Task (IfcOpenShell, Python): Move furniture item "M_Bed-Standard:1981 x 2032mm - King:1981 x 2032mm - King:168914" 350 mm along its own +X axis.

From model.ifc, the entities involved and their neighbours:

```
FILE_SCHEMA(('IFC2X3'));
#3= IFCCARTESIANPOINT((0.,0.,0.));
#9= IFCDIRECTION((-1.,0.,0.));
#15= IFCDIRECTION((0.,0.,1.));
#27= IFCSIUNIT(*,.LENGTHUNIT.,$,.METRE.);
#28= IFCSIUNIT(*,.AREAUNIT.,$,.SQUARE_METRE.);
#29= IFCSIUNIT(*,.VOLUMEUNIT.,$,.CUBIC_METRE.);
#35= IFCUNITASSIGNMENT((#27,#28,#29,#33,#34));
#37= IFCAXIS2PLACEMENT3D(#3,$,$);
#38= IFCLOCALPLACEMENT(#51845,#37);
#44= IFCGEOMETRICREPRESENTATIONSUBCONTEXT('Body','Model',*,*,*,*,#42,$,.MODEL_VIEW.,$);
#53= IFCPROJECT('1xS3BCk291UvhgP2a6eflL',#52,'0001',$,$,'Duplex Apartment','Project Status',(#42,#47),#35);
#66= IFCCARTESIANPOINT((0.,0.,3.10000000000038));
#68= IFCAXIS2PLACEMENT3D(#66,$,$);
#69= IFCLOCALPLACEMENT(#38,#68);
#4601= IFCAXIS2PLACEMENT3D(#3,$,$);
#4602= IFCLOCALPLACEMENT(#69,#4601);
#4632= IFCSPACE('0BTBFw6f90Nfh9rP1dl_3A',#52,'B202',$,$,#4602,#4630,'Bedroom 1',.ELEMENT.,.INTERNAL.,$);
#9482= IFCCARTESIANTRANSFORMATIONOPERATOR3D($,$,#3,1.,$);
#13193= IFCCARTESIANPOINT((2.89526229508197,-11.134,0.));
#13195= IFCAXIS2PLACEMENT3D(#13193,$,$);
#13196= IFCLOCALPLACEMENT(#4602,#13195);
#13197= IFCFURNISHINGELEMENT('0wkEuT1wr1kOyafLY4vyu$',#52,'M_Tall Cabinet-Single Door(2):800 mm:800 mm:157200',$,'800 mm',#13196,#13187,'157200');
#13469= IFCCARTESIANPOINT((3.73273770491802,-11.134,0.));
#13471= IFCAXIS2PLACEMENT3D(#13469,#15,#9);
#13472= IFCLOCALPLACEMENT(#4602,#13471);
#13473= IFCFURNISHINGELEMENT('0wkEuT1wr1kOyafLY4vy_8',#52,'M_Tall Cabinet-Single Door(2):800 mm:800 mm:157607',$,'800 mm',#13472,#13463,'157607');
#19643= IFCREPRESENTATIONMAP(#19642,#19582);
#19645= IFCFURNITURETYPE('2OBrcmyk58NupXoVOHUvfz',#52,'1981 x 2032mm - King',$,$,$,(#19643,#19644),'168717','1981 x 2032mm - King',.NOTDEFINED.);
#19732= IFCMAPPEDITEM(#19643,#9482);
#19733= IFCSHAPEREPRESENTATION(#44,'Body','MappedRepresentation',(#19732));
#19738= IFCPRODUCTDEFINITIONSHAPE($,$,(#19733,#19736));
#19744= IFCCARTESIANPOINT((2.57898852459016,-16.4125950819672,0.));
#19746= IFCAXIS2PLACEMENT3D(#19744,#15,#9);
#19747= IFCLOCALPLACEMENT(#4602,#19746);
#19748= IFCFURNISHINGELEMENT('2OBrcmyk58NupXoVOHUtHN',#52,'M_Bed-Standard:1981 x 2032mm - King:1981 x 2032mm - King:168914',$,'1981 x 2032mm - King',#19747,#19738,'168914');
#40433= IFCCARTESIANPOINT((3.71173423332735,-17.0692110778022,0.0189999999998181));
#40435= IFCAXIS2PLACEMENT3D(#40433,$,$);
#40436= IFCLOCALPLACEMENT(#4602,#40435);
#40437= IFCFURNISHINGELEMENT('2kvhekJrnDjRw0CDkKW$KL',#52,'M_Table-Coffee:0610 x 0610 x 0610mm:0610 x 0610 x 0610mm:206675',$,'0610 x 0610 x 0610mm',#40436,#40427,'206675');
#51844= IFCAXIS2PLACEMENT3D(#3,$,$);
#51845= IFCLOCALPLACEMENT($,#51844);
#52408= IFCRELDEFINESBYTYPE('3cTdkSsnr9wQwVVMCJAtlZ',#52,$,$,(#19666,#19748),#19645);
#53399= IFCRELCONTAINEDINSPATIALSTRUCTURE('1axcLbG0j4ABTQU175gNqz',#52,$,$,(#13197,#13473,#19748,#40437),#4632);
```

```python
import ifcopenshell
import ifcopenshell.api.geometry
import ifcopenshell.util.placement
import ifcopenshell.util.unit

model = ifcopenshell.open("model.ifc")
unit_scale = ifcopenshell.util.unit.calculate_unit_scale(model)

item = model.by_id(19748)
matrix = ifcopenshell.util.placement.get_local_placement(item.ObjectPlacement)
matrix[:3, 3] += matrix[:3, 0] * 0.35 / unit_scale
ifcopenshell.api.geometry.edit_object_placement(model, product=item, matrix=matrix, is_si=False)

print(ifcopenshell.util.placement.get_local_placement(item.ObjectPlacement).round(3) + 0.0)

model.write("model-out.ifc")
```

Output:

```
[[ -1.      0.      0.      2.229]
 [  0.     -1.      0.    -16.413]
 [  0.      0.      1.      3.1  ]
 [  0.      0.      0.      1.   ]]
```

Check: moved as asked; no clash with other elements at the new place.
